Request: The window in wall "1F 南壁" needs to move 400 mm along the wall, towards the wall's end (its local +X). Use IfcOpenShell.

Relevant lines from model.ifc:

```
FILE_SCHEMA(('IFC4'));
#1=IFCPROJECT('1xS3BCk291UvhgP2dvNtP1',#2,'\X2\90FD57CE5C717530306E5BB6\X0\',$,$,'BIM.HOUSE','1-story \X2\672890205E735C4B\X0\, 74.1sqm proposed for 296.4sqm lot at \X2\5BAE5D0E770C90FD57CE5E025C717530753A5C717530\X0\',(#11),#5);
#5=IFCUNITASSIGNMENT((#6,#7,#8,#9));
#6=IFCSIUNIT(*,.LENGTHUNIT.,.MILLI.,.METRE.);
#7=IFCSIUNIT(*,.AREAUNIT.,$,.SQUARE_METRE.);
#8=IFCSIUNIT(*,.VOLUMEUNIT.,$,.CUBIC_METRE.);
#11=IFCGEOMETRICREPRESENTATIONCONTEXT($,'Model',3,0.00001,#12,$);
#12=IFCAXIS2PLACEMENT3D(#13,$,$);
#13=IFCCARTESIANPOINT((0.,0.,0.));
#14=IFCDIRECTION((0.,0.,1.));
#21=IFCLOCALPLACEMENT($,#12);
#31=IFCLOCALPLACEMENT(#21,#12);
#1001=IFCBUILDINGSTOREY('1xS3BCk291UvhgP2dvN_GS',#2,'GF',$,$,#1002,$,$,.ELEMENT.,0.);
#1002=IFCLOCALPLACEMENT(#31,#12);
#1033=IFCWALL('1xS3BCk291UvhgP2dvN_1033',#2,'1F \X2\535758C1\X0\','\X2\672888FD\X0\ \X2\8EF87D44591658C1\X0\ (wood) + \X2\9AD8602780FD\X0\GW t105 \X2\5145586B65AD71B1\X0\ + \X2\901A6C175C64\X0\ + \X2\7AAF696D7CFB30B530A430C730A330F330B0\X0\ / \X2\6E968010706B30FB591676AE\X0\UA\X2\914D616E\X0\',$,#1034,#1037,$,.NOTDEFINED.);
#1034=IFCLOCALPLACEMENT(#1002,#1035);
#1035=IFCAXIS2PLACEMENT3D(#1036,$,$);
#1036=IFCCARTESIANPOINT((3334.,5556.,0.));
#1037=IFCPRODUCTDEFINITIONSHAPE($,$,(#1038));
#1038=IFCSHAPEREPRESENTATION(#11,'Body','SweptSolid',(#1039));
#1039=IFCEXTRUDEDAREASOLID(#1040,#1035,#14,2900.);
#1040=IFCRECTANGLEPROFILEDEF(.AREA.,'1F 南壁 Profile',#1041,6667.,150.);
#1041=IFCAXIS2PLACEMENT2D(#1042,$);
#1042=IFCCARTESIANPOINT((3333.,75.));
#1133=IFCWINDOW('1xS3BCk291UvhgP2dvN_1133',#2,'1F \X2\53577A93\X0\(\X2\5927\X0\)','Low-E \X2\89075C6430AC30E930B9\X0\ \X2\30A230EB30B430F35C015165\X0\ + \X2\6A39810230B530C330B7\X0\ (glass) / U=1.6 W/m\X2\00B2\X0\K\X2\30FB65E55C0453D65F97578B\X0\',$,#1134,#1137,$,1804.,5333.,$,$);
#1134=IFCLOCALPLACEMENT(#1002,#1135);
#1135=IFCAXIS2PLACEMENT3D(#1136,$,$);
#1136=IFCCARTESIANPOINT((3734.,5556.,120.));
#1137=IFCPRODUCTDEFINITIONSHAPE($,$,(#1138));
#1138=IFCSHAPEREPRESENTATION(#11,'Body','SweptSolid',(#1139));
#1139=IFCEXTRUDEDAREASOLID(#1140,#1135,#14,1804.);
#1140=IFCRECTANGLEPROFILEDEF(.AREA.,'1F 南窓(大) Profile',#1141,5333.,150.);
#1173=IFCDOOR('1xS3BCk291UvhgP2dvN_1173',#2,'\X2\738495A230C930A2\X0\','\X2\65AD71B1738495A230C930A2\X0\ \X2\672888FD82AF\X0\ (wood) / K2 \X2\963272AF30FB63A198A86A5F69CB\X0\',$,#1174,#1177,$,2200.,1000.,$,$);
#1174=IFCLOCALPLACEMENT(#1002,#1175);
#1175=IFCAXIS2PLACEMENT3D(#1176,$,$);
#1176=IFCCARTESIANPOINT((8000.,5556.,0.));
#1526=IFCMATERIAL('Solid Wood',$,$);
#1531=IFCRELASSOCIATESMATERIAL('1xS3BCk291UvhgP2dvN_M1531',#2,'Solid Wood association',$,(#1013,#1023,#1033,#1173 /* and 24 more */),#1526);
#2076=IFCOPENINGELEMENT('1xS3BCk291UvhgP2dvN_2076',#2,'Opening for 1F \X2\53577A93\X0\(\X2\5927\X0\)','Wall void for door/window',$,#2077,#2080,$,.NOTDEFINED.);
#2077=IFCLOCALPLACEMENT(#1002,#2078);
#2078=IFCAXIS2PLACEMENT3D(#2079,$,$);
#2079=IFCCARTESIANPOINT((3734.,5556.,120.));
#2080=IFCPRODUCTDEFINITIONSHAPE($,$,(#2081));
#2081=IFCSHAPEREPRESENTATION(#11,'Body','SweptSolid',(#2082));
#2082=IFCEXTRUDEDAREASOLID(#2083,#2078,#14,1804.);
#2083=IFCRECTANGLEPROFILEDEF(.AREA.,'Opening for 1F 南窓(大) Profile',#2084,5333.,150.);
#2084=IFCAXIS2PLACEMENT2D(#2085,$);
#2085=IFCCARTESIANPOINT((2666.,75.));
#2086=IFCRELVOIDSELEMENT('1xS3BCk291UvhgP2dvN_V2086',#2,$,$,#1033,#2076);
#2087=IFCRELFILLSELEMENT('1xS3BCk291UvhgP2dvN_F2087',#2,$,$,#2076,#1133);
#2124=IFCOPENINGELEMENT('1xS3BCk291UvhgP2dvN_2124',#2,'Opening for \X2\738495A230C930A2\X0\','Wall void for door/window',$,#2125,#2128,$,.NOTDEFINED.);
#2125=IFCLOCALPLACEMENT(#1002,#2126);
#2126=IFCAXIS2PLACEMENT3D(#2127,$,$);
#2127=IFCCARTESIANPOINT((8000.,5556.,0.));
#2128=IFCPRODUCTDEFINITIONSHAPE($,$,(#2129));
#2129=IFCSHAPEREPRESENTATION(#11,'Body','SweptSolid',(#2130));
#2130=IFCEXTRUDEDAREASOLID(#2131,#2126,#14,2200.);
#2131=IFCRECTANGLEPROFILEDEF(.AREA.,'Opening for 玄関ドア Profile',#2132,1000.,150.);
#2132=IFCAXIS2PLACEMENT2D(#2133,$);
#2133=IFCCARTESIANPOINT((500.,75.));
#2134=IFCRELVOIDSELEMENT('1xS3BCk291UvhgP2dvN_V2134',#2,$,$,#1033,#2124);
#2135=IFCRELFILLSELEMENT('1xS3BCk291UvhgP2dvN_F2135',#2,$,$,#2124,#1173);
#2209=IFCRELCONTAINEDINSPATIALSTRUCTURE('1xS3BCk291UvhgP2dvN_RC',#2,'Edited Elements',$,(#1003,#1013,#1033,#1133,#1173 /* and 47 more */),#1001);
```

```python
import ifcopenshell
import ifcopenshell.api.geometry
import ifcopenshell.util.placement

model = ifcopenshell.open("model.ifc")

window = model.by_id(1133)
opening = window.FillsVoids[0].RelatingOpeningElement
wall = opening.VoidsElements[0].RelatingBuildingElement

wall_matrix = ifcopenshell.util.placement.get_local_placement(wall.ObjectPlacement)
shift = wall_matrix[:3, 0] * 400.0
before = ifcopenshell.util.placement.get_local_placement(window.ObjectPlacement)[:3, 3].copy()

# The window is not placed relative to its opening, so move both.
for product in (opening, window):
    matrix = ifcopenshell.util.placement.get_local_placement(product.ObjectPlacement)
    matrix[:3, 3] += shift
    ifcopenshell.api.geometry.edit_object_placement(model, product=product, matrix=matrix, is_si=False)

after = ifcopenshell.util.placement.get_local_placement(window.ObjectPlacement)[:3, 3]
print("window moved by", (after - before).round(3) + 0.0)

model.write("model_edited.ifc")
```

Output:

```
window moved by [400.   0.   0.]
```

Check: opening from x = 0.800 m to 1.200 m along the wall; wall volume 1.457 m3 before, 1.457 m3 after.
